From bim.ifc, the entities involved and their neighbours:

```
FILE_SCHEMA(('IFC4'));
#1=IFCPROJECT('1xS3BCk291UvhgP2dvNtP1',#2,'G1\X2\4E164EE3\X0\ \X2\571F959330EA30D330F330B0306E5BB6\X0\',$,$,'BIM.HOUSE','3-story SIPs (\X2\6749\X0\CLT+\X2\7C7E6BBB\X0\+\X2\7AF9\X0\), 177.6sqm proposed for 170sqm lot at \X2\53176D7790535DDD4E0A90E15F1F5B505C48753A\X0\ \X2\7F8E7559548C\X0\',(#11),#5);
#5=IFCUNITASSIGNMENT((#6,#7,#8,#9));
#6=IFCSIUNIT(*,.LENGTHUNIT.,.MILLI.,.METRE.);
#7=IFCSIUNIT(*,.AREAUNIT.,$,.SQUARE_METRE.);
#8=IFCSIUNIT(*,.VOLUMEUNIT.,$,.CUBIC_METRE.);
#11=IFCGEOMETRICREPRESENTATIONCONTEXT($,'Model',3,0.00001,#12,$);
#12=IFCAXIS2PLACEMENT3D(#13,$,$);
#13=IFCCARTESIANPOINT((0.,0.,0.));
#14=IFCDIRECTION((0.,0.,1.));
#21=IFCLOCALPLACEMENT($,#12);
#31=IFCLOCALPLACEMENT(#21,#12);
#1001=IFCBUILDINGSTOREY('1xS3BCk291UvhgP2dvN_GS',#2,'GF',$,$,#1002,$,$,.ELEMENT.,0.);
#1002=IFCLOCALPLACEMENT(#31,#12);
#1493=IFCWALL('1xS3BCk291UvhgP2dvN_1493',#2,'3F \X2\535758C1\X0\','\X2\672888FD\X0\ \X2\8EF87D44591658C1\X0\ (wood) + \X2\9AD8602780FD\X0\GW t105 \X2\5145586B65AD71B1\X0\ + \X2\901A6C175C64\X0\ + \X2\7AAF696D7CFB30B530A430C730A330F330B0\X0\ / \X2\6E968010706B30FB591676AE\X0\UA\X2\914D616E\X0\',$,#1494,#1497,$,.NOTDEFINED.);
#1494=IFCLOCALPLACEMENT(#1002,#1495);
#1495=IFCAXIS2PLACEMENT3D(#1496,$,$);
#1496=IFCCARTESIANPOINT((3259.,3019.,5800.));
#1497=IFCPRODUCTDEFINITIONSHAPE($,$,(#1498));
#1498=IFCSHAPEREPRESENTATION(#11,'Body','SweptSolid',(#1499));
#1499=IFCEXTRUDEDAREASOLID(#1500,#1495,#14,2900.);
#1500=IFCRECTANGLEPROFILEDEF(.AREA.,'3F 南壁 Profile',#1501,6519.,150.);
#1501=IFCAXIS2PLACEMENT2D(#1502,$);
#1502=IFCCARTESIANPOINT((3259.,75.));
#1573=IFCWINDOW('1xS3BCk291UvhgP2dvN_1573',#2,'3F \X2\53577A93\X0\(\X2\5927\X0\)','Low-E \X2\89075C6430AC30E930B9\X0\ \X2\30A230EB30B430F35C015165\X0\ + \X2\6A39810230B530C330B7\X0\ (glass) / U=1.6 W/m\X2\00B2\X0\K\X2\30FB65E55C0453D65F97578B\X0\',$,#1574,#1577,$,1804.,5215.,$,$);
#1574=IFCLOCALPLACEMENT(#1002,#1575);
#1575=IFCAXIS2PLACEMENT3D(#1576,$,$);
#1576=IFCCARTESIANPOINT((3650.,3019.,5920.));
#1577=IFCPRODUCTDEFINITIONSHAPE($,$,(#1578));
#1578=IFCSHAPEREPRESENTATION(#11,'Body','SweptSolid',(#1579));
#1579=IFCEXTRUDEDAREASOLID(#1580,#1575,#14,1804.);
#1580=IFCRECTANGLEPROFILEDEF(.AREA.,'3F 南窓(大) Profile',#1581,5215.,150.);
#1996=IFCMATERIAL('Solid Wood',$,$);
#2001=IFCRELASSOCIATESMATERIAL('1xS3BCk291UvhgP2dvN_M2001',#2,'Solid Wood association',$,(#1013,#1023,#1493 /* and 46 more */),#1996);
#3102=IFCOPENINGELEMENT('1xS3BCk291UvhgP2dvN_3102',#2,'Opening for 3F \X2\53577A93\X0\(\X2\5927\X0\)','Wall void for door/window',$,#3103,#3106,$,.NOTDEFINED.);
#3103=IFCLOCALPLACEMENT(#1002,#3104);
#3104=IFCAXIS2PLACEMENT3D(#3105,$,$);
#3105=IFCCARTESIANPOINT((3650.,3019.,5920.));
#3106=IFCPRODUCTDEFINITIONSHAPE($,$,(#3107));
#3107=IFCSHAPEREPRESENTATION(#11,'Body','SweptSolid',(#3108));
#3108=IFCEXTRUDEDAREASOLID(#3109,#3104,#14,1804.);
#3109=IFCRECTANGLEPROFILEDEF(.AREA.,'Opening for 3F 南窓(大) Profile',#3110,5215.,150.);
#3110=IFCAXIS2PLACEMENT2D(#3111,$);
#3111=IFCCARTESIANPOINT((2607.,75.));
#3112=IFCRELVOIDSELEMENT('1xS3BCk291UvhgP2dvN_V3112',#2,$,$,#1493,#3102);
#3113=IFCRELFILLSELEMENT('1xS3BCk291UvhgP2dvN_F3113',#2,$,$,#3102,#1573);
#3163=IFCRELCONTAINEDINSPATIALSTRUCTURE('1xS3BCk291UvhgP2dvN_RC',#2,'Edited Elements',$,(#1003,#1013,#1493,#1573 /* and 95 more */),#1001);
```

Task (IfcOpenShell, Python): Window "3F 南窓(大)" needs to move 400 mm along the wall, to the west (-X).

```python
import ifcopenshell
import ifcopenshell.api.geometry
import ifcopenshell.util.placement
import ifcopenshell.util.unit

model = ifcopenshell.open("bim.ifc")
unit_scale = ifcopenshell.util.unit.calculate_unit_scale(model)

window = model.by_guid("1xS3BCk291UvhgP2dvN_1573")
opening = window.FillsVoids[0].RelatingOpeningElement
wall = opening.VoidsElements[0].RelatingBuildingElement

wall_matrix = ifcopenshell.util.placement.get_local_placement(wall.ObjectPlacement)
shift = wall_matrix[:3, 0] * -0.4 / unit_scale
before = ifcopenshell.util.placement.get_local_placement(window.ObjectPlacement)[:3, 3].copy()

# The window is not placed relative to its opening, so move both.
for product in (opening, window):
    matrix = ifcopenshell.util.placement.get_local_placement(product.ObjectPlacement)
    matrix[:3, 3] += shift
    ifcopenshell.api.geometry.edit_object_placement(model, product=product, matrix=matrix, is_si=False)

after = ifcopenshell.util.placement.get_local_placement(window.ObjectPlacement)[:3, 3]
print("window moved by", (after - before).round(3) + 0.0)

model.write("bim_rev.ifc")
```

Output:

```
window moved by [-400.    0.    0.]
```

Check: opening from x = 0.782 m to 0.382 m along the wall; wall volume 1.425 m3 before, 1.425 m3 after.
